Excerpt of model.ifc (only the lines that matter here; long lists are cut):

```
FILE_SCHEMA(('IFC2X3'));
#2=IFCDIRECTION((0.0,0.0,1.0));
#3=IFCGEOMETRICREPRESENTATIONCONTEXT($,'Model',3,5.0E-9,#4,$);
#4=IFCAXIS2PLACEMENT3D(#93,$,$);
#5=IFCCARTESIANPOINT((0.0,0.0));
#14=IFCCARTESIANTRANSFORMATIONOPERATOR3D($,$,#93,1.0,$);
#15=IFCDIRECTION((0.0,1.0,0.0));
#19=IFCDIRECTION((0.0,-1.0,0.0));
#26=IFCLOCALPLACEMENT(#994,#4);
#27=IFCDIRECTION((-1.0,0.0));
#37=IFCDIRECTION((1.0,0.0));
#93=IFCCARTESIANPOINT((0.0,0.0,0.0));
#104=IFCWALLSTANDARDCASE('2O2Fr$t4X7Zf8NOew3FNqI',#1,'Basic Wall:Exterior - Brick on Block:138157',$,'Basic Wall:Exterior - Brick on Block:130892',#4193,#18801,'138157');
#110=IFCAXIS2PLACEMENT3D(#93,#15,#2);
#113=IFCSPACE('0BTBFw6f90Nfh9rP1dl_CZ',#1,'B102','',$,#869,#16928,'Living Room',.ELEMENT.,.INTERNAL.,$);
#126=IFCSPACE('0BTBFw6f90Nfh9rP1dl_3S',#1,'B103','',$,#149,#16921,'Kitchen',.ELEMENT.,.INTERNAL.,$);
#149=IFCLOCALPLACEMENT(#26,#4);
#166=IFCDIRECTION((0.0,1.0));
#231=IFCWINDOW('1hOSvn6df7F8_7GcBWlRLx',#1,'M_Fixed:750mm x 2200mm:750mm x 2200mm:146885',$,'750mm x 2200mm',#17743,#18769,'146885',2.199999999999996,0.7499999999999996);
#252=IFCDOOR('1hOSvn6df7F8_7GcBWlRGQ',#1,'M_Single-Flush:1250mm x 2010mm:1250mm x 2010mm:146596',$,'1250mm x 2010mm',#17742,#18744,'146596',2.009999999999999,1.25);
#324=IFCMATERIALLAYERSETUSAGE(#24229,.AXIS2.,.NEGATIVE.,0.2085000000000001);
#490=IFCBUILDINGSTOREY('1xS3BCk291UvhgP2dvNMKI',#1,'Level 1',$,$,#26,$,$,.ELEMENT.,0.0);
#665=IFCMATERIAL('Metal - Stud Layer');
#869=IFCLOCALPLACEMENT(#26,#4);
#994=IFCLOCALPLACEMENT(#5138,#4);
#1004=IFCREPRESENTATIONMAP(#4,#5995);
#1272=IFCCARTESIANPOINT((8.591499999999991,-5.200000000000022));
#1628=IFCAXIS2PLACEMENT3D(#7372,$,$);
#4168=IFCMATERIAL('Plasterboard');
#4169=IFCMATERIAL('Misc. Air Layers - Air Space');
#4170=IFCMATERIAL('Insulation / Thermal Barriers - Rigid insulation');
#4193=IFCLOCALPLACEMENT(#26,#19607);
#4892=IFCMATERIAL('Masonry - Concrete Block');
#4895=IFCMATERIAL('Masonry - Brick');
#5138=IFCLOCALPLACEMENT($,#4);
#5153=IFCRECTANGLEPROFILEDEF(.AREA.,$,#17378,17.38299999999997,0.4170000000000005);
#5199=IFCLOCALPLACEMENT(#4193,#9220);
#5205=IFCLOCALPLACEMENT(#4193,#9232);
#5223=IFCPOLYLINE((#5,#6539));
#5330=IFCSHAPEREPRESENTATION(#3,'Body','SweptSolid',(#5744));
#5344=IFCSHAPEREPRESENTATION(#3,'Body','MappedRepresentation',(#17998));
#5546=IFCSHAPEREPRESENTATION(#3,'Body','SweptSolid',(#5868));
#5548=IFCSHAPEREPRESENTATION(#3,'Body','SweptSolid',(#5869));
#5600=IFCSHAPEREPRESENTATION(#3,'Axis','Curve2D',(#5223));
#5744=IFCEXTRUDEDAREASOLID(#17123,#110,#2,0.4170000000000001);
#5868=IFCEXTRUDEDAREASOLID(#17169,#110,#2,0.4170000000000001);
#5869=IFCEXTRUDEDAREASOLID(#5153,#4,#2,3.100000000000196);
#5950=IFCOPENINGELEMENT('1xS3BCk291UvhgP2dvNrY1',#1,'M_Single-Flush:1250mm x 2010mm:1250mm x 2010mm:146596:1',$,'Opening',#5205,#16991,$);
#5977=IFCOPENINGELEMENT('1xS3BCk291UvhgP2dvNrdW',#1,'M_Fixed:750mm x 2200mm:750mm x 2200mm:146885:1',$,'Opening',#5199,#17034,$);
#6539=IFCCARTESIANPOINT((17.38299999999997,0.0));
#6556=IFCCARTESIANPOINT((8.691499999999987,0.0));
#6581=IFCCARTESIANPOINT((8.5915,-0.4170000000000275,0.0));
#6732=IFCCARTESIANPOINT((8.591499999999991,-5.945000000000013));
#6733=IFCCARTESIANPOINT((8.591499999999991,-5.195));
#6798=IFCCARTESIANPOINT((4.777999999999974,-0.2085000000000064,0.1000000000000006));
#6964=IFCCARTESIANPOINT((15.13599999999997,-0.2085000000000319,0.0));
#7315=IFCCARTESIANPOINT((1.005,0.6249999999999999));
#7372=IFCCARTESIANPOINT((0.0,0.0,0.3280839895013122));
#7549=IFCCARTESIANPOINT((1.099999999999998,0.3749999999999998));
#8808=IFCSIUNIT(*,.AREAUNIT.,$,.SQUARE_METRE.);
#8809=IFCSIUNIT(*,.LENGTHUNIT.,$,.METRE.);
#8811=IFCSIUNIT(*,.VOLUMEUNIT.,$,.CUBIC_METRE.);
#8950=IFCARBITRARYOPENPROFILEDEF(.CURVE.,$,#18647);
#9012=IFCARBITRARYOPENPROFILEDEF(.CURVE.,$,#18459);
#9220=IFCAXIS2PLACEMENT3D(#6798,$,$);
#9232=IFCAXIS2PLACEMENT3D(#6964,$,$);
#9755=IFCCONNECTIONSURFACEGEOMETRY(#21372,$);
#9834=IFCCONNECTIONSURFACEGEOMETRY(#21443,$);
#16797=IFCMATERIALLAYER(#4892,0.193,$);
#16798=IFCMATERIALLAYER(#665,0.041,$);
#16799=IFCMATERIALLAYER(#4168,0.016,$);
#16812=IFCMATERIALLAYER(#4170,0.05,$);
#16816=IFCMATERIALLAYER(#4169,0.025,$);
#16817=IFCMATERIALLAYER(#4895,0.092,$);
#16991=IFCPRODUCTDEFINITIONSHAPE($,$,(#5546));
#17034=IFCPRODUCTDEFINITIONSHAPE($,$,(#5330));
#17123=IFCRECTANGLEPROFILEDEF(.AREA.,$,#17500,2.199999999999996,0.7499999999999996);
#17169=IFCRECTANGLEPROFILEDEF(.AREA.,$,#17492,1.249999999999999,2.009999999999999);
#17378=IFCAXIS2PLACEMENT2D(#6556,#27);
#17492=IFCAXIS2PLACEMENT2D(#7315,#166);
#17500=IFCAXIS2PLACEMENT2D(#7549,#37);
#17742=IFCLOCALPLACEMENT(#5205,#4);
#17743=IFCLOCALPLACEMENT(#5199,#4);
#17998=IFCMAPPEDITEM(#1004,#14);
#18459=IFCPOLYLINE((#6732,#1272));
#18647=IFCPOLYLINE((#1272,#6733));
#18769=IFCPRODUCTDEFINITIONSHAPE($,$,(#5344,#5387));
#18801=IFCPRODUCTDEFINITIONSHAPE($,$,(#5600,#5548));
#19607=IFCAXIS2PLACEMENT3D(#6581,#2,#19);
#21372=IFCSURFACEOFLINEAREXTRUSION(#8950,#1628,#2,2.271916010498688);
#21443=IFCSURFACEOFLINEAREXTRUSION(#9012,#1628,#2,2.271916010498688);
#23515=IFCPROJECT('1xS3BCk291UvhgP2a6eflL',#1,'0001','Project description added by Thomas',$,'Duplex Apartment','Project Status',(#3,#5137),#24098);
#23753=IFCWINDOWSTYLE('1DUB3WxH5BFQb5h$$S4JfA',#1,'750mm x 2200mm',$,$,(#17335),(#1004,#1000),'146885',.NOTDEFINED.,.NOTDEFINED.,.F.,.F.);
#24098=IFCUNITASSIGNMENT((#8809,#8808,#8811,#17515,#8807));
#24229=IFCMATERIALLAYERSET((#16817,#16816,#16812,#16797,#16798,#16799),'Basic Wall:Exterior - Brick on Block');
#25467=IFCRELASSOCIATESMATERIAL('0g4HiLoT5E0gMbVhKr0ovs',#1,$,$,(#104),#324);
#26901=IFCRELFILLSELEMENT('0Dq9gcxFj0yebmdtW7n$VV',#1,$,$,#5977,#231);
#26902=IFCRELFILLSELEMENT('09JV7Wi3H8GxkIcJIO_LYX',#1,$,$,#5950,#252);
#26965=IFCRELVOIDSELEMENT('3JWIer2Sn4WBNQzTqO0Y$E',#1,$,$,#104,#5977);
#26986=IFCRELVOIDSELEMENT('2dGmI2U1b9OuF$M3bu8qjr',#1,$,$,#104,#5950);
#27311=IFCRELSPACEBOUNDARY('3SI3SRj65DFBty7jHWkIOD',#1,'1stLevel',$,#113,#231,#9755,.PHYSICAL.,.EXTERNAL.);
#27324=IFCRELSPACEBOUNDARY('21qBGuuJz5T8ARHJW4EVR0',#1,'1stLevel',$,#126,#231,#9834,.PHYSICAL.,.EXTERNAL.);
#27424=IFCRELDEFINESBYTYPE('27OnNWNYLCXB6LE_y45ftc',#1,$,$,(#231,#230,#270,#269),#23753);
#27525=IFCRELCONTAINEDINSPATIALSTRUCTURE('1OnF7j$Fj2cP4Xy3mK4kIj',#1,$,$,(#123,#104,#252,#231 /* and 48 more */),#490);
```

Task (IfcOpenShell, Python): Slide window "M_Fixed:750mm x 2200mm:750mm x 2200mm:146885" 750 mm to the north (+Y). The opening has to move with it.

```python
import numpy as np
import ifcopenshell
import ifcopenshell.api.geometry
import ifcopenshell.util.placement
import ifcopenshell.util.unit

model = ifcopenshell.open("model.ifc")
unit_scale = ifcopenshell.util.unit.calculate_unit_scale(model)

window = model.by_guid("1hOSvn6df7F8_7GcBWlRLx")
opening = window.FillsVoids[0].RelatingOpeningElement
wall = opening.VoidsElements[0].RelatingBuildingElement

wall_matrix = ifcopenshell.util.placement.get_local_placement(wall.ObjectPlacement)
shift = wall_matrix[:3, 0] * -0.75 / unit_scale
before = ifcopenshell.util.placement.get_local_placement(window.ObjectPlacement)[:3, 3].copy()

# The window is placed relative to its opening, so it follows when the opening moves.
matrix = ifcopenshell.util.placement.get_local_placement(opening.ObjectPlacement)
matrix[:3, 3] += shift
ifcopenshell.api.geometry.edit_object_placement(
    model, product=opening, matrix=matrix, is_si=False, should_transform_children=True
)

# Space boundary surfaces are stored in each space's coordinates; move them too.
for rel in window.ProvidesBoundaries:
    if not rel.ConnectionGeometry:
        continue
    surface = rel.ConnectionGeometry.SurfaceOnRelatingElement
    space_matrix = ifcopenshell.util.placement.get_local_placement(rel.RelatingSpace.ObjectPlacement)
    point = np.array(surface.Position.Location.Coordinates) + space_matrix[:3, :3].T @ shift
    surface.Position = model.createIfcAxis2Placement3D(
        model.createIfcCartesianPoint(point.tolist()), surface.Position.Axis, surface.Position.RefDirection
    )

after = ifcopenshell.util.placement.get_local_placement(window.ObjectPlacement)[:3, 3]
print("window moved by", (after - before).round(3) + 0.0)

model.write("model_updated.ifc")
```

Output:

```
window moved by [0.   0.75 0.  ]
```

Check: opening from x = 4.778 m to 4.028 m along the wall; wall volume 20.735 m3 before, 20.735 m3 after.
